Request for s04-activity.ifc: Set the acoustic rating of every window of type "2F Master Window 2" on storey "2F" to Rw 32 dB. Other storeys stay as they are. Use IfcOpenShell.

First a look at what the model holds.

```python
import ifcopenshell
import ifcopenshell.util.element

model = ifcopenshell.open("s04-activity.ifc")
print(model.schema)
storey = next(s for s in model.by_type("IfcBuildingStorey") if s.Name == "2F")
windows = [e for e in ifcopenshell.util.element.get_decomposition(storey) if e.is_a("IfcWindow")]
seen = {}
for e in windows:
    element_type = ifcopenshell.util.element.get_type(e)
    key = (element_type.Name if element_type != e and element_type else None, ifcopenshell.util.element.get_pset(e, "Pset_WindowCommon", "AcousticRating"))
    seen[key] = seen.get(key, 0) + 1
for (name, value), count in sorted(seen.items(), key=str):
    print(count, "x", name, "|", value)
```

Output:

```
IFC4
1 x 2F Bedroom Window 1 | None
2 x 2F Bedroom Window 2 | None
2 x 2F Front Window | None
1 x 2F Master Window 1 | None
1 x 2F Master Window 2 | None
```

```python
import ifcopenshell
import ifcopenshell.api.pset
import ifcopenshell.util.element

model = ifcopenshell.open("s04-activity.ifc")

storey = next(s for s in model.by_type("IfcBuildingStorey") if s.Name == "2F")
windows = [e for e in ifcopenshell.util.element.get_decomposition(storey) if e.is_a("IfcWindow")]

count = 0
for e in windows:
    element_type = ifcopenshell.util.element.get_type(e)
    if element_type in (None, e) or element_type.Name != "2F Master Window 2":
        continue
    # add_pset returns the element's existing set when there is one.
    pset = ifcopenshell.api.pset.add_pset(model, product=e, name="Pset_WindowCommon")
    ifcopenshell.api.pset.edit_pset(model, pset=pset, properties={"AcousticRating": "Rw 32 dB"})
    count += 1

print(count, "windows updated")

model.write("s04-activity-out.ifc")
```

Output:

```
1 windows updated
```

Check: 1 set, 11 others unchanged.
